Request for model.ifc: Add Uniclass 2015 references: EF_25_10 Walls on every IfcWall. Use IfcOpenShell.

First a look at what the model holds.

```python
import ifcopenshell

model = ifcopenshell.open("model.ifc")
print(model.schema)
print("classifications:", [c.Name for c in model.by_type("IfcClassification")])
for ifc_class in ("IfcDoor", "IfcRoof", "IfcStair", "IfcWall", "IfcWindow"):
    print(ifc_class, len(model.by_type(ifc_class)))
```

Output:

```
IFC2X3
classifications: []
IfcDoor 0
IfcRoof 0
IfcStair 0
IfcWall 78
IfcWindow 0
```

```python
import ifcopenshell
import ifcopenshell.api.classification

model = ifcopenshell.open("model.ifc")

# IFC2X3 requires Source and Edition and has no link from the project to the system.
system = model.create_entity("IfcClassification", Source="NBS", Edition="2015", Name="Uniclass 2015")

codes = {
    "IfcWall": ("EF_25_10", "Walls"),
}
for ifc_class, (code, name) in codes.items():
    products = model.by_type(ifc_class)
    ifcopenshell.api.classification.add_reference(
        model, products=products, classification=system, identification=code, name=name
    )
    print(code, len(products))

model.write("model-out.ifc")
```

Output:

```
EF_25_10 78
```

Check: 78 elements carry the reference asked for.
